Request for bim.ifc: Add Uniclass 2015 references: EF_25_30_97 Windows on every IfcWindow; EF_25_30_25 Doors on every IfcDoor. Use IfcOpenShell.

First a look at what the model holds.

```python
import ifcopenshell

model = ifcopenshell.open("bim.ifc")
print(model.schema)
print("classifications:", [c.Name for c in model.by_type("IfcClassification")])
for ifc_class in ("IfcDoor", "IfcRoof", "IfcStair", "IfcWall", "IfcWindow"):
    print(ifc_class, len(model.by_type(ifc_class)))
```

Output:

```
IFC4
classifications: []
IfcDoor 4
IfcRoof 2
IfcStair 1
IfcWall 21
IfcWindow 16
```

```python
import ifcopenshell
import ifcopenshell.api.classification

model = ifcopenshell.open("bim.ifc")

system = ifcopenshell.api.classification.add_classification(model, classification="Uniclass 2015")

codes = {
    "IfcWindow": ("EF_25_30_97", "Windows"),
    "IfcDoor": ("EF_25_30_25", "Doors"),
}
for ifc_class, (code, name) in codes.items():
    products = model.by_type(ifc_class)
    ifcopenshell.api.classification.add_reference(
        model, products=products, classification=system, identification=code, name=name
    )
    print(code, len(products))

model.write("bim_v2.ifc")
```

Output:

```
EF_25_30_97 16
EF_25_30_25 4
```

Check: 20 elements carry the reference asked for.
